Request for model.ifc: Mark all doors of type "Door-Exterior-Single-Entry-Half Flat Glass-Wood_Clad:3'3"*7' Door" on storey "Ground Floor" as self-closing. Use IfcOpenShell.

First a look at what the model holds.

```python
import ifcopenshell
import ifcopenshell.util.element

model = ifcopenshell.open("model.ifc")
print(model.schema)
storey = next(s for s in model.by_type("IfcBuildingStorey") if s.Name == "Ground Floor")
doors = [e for e in ifcopenshell.util.element.get_decomposition(storey) if e.is_a("IfcDoor")]
seen = {}
for e in doors:
    element_type = ifcopenshell.util.element.get_type(e)
    key = (element_type.Name if element_type != e and element_type else None, ifcopenshell.util.element.get_pset(e, "Pset_DoorCommon", "SelfClosing"))
    seen[key] = seen.get(key, 0) + 1
for (name, value), count in sorted(seen.items(), key=str):
    print(count, "x", name, "|", value)
```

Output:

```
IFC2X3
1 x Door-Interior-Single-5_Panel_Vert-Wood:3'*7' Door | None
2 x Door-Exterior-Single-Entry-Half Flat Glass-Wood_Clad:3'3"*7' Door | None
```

```python
import ifcopenshell
import ifcopenshell.api.pset
import ifcopenshell.util.element

model = ifcopenshell.open("model.ifc")

storey = next(s for s in model.by_type("IfcBuildingStorey") if s.Name == "Ground Floor")
doors = [e for e in ifcopenshell.util.element.get_decomposition(storey) if e.is_a("IfcDoor")]

count = 0
for e in doors:
    element_type = ifcopenshell.util.element.get_type(e)
    if element_type in (None, e) or element_type.Name != 'Door-Exterior-Single-Entry-Half Flat Glass-Wood_Clad:3\'3"*7\' Door':
        continue
    # add_pset returns the element's existing set when there is one.
    pset = ifcopenshell.api.pset.add_pset(model, product=e, name="Pset_DoorCommon")
    ifcopenshell.api.pset.edit_pset(model, pset=pset, properties={"SelfClosing": True})
    count += 1

print(count, "doors updated")

model.write("model_updated.ifc")
```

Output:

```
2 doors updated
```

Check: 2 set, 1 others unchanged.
